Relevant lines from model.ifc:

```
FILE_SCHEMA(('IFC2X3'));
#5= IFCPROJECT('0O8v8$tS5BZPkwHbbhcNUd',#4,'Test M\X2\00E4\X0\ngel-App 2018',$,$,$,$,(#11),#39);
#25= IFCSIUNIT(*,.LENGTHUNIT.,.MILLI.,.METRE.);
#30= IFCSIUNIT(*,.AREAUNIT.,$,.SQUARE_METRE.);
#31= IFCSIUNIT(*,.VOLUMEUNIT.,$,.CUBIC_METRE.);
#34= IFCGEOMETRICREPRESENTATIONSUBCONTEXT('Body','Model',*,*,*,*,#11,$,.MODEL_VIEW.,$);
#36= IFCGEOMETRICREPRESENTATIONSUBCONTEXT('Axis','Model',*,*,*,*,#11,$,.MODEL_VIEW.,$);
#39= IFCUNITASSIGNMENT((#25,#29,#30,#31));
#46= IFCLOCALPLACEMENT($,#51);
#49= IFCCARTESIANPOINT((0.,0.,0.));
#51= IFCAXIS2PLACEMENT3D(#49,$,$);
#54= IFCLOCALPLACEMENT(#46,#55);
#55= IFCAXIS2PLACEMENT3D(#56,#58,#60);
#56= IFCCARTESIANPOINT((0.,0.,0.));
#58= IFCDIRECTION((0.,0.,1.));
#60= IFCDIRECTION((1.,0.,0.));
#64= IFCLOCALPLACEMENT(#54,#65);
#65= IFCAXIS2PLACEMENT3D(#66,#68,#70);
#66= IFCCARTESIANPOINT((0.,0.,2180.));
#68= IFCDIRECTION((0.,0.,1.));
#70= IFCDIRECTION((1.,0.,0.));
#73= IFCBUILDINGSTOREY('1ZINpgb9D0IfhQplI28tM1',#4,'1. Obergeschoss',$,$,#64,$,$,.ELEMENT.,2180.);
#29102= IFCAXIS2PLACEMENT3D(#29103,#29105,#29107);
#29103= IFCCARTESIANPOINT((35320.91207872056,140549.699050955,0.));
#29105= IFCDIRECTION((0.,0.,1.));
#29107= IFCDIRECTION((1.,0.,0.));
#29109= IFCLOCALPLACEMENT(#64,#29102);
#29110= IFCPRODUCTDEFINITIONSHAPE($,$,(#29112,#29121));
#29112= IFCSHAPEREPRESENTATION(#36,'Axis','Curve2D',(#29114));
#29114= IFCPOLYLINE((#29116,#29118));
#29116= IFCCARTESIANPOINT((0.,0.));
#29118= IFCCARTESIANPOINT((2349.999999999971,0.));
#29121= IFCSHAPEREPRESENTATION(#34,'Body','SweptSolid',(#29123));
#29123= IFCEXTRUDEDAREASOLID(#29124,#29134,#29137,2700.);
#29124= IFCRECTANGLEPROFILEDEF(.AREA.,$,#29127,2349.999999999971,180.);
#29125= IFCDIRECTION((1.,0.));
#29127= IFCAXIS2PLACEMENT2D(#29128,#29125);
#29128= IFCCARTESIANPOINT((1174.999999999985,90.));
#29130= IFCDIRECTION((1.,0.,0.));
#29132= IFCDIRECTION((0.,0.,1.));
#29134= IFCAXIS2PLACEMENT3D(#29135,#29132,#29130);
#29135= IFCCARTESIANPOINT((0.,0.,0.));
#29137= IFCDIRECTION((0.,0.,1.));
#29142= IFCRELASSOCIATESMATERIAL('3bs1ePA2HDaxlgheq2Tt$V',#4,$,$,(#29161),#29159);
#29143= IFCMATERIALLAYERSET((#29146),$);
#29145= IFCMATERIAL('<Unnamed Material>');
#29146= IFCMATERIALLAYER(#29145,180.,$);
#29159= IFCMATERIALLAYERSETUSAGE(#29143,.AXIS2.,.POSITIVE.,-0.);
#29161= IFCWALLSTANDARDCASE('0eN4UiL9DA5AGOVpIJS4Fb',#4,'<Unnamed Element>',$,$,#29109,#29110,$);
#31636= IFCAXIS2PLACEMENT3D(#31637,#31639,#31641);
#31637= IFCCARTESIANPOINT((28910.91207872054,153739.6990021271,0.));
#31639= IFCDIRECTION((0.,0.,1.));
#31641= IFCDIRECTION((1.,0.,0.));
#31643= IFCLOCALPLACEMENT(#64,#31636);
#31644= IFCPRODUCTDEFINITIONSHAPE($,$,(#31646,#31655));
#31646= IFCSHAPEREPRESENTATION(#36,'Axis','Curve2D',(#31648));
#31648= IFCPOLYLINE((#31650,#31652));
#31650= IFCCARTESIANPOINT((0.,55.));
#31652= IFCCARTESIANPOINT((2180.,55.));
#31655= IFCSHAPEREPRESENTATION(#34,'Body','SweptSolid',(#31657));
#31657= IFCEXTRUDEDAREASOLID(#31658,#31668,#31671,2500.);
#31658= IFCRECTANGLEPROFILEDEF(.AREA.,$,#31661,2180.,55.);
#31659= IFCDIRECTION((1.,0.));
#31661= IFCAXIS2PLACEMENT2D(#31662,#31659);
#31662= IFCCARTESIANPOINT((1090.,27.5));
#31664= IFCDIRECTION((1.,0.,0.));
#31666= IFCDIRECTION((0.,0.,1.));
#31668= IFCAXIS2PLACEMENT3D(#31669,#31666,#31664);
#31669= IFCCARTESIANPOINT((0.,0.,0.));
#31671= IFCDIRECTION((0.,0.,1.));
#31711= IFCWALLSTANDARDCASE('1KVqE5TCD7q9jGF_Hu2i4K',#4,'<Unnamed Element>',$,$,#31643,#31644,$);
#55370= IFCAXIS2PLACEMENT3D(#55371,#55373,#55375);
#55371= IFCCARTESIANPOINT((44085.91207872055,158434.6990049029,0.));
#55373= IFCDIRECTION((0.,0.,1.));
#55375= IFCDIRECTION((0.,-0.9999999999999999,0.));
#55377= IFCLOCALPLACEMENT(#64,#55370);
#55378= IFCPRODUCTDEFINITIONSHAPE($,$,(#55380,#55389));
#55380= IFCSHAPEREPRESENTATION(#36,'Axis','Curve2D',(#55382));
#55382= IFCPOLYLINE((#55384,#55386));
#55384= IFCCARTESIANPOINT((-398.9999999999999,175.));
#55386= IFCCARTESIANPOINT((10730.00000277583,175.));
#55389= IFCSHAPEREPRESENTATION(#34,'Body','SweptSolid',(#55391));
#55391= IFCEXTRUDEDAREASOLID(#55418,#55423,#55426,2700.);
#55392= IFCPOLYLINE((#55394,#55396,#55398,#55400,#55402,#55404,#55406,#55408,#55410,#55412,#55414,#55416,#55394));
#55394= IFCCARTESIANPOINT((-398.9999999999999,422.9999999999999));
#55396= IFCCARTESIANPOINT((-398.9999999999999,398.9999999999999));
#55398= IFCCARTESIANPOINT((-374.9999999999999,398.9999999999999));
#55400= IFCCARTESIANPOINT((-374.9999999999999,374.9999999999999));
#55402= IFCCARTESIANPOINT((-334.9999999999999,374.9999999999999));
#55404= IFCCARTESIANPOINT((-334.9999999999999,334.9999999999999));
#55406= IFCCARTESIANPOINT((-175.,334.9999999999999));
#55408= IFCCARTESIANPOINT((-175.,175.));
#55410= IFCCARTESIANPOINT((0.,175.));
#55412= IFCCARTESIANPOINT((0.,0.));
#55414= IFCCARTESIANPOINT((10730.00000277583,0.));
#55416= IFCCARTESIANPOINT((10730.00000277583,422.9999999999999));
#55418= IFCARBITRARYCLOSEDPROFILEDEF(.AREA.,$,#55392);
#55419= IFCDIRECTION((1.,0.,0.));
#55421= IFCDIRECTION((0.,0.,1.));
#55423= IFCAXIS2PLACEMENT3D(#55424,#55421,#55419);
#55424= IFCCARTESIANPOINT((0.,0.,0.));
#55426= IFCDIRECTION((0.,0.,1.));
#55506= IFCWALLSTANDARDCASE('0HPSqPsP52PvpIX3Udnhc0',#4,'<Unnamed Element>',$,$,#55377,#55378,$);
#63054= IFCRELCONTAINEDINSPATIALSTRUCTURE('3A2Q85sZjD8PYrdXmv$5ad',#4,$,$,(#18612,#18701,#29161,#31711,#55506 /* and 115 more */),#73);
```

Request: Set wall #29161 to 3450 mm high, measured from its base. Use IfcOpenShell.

```python
import ifcopenshell
import ifcopenshell.geom
import ifcopenshell.util.representation
import ifcopenshell.util.shape

model = ifcopenshell.open("model.ifc")
settings = ifcopenshell.geom.settings()


def volume(element):
    """Net volume in cubic metres, openings subtracted."""
    shape = ifcopenshell.geom.create_shape(settings, element)
    return ifcopenshell.util.shape.get_volume(shape.geometry)


wall = model.by_guid("0eN4UiL9DA5AGOVpIJS4Fb")
before = volume(wall)

body = ifcopenshell.util.representation.get_representation(wall, "Model", "Body")
solid = body.Items[0]
old_height = solid.Depth
solid.Depth = 3450.0
after = volume(wall)

print(f"height {old_height:g} -> {solid.Depth:g}, volume {before:.3f} -> {after:.3f} m3")

model.write("model-out.ifc")
```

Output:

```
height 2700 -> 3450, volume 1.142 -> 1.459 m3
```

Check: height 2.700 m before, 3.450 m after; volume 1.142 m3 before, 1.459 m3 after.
